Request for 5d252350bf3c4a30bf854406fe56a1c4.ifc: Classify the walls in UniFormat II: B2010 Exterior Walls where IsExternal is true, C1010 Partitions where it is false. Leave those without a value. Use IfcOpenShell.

First a look at what the model holds.

```python
import ifcopenshell
import ifcopenshell.util.element

model = ifcopenshell.open("5d252350bf3c4a30bf854406fe56a1c4.ifc")
print(model.schema)
print("classifications:", [c.Name for c in model.by_type("IfcClassification")])
values = [ifcopenshell.util.element.get_pset(e, "Pset_WallCommon", "IsExternal") for e in model.by_type("IfcWall")]
for value in (True, False, None):
    print("IsExternal", value, values.count(value))
```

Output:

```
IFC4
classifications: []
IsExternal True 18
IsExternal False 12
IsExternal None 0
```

```python
import ifcopenshell
import ifcopenshell.api.classification
import ifcopenshell.util.element

model = ifcopenshell.open("5d252350bf3c4a30bf854406fe56a1c4.ifc")

system = ifcopenshell.api.classification.add_classification(model, classification="UniFormat II")

walls = model.by_type("IfcWall")
external = {e: ifcopenshell.util.element.get_pset(e, "Pset_WallCommon", "IsExternal") for e in walls}
for flag, code, name in ((True, "B2010", "Exterior Walls"), (False, "C1010", "Partitions")):
    products = [e for e in walls if external[e] is flag]
    ifcopenshell.api.classification.add_reference(
        model, products=products, classification=system, identification=code, name=name
    )
    print(code, len(products))

model.write("5d252350bf3c4a30bf854406fe56a1c4_updated.ifc")
```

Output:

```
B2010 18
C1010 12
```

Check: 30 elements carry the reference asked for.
